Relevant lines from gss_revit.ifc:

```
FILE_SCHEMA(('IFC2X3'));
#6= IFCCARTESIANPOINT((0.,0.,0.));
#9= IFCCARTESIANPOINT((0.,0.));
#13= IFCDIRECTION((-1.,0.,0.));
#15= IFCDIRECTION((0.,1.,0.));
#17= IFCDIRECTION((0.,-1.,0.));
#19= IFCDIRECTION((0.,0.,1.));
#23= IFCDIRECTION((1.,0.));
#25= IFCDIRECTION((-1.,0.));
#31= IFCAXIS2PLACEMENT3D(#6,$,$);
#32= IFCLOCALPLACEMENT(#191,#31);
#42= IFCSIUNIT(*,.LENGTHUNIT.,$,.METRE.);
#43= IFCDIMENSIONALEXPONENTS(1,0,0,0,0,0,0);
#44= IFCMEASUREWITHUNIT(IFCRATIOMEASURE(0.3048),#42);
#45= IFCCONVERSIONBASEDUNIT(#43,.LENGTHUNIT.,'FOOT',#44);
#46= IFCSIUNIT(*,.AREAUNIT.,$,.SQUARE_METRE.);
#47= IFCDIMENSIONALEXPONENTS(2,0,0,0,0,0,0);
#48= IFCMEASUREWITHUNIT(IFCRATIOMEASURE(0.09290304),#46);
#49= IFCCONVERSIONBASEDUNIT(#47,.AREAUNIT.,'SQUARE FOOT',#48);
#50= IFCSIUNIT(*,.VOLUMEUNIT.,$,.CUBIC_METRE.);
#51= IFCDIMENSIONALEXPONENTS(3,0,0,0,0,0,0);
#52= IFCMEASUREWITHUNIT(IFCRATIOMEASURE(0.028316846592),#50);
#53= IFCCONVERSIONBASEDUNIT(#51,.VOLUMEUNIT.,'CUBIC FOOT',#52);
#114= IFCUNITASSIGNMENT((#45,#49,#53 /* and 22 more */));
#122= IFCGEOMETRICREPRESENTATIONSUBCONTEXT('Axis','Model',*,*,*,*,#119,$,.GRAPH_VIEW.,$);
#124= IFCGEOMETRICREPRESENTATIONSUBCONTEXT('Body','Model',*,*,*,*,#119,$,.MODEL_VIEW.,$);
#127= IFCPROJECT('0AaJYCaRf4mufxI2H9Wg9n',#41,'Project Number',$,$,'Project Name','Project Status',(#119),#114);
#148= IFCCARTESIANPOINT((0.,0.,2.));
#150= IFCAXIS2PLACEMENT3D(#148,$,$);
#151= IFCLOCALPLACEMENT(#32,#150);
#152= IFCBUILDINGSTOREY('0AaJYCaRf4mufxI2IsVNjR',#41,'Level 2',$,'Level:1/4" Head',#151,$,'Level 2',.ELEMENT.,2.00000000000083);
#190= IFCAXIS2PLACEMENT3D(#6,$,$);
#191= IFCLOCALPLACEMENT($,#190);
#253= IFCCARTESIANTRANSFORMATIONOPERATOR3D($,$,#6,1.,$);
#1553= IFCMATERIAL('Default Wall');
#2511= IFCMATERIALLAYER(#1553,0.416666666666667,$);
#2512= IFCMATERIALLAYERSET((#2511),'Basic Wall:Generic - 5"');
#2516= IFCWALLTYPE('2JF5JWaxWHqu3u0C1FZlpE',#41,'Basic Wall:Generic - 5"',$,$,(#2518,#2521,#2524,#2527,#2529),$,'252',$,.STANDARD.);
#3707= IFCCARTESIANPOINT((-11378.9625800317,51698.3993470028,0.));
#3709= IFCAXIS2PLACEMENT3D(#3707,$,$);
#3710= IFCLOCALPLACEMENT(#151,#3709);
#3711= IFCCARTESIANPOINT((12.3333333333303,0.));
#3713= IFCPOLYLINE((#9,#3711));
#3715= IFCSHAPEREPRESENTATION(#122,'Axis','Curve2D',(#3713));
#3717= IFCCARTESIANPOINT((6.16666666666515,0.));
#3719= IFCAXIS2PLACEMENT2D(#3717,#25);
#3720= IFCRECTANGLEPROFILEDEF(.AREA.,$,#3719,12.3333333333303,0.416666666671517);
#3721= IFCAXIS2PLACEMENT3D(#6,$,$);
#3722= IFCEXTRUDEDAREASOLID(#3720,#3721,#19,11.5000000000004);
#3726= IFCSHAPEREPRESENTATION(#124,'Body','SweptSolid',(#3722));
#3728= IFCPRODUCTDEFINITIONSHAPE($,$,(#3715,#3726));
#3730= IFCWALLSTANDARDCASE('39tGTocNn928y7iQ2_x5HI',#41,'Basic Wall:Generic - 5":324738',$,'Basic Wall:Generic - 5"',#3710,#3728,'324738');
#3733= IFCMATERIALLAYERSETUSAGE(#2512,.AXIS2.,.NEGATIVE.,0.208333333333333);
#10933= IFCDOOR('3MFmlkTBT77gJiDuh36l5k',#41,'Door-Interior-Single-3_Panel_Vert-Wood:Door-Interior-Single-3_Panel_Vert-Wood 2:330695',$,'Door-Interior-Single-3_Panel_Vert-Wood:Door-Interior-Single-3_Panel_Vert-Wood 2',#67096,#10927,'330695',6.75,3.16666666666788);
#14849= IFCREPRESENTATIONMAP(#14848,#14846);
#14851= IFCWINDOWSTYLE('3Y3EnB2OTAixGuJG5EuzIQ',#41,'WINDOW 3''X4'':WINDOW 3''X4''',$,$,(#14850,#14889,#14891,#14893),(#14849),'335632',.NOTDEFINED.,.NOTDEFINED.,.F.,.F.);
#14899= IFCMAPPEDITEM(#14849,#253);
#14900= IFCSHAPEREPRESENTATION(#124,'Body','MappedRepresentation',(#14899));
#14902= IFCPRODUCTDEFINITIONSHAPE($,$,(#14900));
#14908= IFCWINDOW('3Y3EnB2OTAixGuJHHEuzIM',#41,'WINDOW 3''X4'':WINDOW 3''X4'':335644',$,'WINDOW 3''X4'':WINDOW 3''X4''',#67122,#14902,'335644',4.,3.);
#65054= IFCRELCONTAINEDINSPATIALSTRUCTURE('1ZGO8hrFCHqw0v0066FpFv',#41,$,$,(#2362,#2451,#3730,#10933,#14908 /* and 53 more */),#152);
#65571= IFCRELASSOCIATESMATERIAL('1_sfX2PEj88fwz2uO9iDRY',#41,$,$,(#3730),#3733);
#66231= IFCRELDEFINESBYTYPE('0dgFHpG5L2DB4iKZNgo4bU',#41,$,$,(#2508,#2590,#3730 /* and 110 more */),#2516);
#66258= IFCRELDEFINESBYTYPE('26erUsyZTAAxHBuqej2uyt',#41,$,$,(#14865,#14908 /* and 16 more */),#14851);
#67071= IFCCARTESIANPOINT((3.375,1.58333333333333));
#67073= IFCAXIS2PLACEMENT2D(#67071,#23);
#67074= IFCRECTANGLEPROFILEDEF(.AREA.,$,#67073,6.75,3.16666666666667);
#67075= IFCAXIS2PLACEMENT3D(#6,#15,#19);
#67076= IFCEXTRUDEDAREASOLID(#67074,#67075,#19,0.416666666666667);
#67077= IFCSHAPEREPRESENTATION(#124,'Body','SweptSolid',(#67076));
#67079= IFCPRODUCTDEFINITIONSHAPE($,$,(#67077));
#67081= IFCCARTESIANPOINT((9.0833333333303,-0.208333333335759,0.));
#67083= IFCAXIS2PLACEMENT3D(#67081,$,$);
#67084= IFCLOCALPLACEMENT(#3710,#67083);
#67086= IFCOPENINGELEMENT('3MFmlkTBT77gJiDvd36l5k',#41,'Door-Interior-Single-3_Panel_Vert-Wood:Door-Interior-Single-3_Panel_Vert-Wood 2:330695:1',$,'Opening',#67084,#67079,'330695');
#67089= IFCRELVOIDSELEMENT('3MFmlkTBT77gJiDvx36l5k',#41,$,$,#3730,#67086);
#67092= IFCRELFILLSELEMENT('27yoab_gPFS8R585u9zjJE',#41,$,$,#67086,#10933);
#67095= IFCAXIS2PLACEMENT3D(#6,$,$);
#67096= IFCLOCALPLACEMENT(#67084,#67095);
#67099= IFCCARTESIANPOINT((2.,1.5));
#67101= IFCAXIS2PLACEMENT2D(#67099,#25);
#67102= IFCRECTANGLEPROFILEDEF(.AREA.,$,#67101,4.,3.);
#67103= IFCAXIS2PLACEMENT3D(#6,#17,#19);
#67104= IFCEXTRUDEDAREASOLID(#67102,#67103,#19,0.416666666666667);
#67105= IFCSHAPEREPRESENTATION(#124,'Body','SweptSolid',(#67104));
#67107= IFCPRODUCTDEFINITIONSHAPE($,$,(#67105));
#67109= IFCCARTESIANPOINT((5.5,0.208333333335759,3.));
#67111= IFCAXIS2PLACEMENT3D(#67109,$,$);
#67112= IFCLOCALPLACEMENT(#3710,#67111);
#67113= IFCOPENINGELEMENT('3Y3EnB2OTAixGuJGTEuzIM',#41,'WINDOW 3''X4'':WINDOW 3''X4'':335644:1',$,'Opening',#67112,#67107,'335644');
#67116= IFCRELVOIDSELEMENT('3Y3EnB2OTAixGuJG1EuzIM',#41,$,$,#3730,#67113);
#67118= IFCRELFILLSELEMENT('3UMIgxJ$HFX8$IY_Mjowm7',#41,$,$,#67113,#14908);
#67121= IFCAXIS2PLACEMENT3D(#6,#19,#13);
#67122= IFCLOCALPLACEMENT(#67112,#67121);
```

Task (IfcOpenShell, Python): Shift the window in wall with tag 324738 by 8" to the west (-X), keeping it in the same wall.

```python
import ifcopenshell
import ifcopenshell.api.geometry
import ifcopenshell.util.placement
import ifcopenshell.util.unit

model = ifcopenshell.open("gss_revit.ifc")
unit_scale = ifcopenshell.util.unit.calculate_unit_scale(model)

window = model.by_guid("3Y3EnB2OTAixGuJHHEuzIM")
opening = window.FillsVoids[0].RelatingOpeningElement
wall = opening.VoidsElements[0].RelatingBuildingElement

wall_matrix = ifcopenshell.util.placement.get_local_placement(wall.ObjectPlacement)
shift = wall_matrix[:3, 0] * -8 * 0.0254 / unit_scale
before = ifcopenshell.util.placement.get_local_placement(window.ObjectPlacement)[:3, 3].copy()

# The window is placed relative to its opening, so it follows when the opening moves.
matrix = ifcopenshell.util.placement.get_local_placement(opening.ObjectPlacement)
matrix[:3, 3] += shift
ifcopenshell.api.geometry.edit_object_placement(
    model, product=opening, matrix=matrix, is_si=False, should_transform_children=True
)

after = ifcopenshell.util.placement.get_local_placement(window.ObjectPlacement)[:3, 3]
print("window moved by", (after - before).round(3) + 0.0)

model.write("gss_revit_edited.ifc")
```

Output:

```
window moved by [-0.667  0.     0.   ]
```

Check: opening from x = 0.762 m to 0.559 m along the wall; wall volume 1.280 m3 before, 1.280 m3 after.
